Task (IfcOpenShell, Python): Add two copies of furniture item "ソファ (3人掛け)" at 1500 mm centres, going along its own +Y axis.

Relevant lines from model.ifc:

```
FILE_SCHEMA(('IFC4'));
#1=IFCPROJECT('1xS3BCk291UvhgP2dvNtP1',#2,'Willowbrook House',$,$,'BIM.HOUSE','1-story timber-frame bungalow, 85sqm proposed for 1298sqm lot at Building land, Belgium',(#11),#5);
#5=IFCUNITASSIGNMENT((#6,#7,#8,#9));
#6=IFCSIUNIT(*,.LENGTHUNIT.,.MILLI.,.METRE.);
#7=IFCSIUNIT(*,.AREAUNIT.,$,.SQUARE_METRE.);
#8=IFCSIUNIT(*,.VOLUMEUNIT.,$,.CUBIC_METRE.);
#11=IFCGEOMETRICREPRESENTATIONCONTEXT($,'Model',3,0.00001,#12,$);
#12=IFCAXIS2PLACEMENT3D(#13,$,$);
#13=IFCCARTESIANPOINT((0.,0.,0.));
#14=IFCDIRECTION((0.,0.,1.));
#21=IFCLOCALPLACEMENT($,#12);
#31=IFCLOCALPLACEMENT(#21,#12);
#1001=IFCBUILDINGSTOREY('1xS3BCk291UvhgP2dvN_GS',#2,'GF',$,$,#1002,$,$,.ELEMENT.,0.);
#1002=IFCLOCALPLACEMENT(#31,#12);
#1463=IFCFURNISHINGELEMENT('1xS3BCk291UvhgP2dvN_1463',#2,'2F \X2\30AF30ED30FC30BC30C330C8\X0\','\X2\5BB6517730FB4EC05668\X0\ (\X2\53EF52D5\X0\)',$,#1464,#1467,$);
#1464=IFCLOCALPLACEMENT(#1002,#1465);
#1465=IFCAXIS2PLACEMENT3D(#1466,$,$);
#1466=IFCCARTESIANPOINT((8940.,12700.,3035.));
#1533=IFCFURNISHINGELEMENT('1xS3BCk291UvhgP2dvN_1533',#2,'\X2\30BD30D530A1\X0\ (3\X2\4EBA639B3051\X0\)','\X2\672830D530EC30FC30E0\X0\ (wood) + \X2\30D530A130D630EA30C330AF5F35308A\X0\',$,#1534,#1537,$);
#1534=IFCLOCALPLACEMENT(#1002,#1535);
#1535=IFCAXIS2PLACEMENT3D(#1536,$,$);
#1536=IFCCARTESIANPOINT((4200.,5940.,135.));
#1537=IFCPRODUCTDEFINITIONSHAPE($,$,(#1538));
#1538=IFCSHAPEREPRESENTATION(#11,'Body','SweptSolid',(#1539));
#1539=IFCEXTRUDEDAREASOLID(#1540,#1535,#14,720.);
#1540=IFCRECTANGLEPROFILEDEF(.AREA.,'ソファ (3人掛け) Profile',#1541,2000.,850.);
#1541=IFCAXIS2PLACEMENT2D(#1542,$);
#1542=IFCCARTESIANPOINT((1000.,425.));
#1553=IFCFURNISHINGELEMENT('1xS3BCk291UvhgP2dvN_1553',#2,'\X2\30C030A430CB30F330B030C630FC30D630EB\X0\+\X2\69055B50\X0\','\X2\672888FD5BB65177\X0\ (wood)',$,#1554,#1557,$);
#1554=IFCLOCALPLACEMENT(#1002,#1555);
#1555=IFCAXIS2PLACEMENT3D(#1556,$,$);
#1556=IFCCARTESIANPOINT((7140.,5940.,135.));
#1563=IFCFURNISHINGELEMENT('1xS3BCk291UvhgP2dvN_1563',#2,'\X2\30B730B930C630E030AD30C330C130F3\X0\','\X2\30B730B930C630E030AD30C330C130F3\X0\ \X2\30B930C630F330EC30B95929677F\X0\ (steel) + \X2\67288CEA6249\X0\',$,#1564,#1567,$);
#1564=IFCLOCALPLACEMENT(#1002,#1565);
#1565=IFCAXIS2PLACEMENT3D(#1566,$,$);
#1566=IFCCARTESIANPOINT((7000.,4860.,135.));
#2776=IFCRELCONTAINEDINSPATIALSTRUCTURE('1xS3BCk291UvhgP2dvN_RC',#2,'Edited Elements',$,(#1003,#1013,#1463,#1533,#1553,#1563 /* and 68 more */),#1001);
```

```python
import ifcopenshell
import ifcopenshell.api.geometry
import ifcopenshell.api.root
import ifcopenshell.util.element
import ifcopenshell.util.placement
import ifcopenshell.util.unit

model = ifcopenshell.open("model.ifc")
unit_scale = ifcopenshell.util.unit.calculate_unit_scale(model)


def reuse_history(source, copy):
    """copy_class also copies each property set's owner history, people and application; keep the originals."""
    for rel in copy.IsDefinedBy:
        if rel.is_a("IfcRelDefinesByProperties") and (history := rel.RelatingPropertyDefinition.OwnerHistory):
            rel.RelatingPropertyDefinition.OwnerHistory = source.OwnerHistory
            ifcopenshell.util.element.remove_deep2(model, history)


source = model.by_id(1533)
base = ifcopenshell.util.placement.get_local_placement(source.ObjectPlacement)
step = base[:3, 1] * 1.5 / unit_scale

for i in range(1, 3):
    copy = ifcopenshell.api.root.copy_class(model, product=source)
    copy.Representation = ifcopenshell.util.element.copy_deep(
        model, source.Representation, exclude=["IfcGeometricRepresentationContext", "IfcRepresentationMap"]
    )
    reuse_history(source, copy)
    matrix = base.copy()
    matrix[:3, 3] += i * step
    print("added at", matrix[:3, 3].round(3) + 0.0)
    ifcopenshell.api.geometry.edit_object_placement(model, product=copy, matrix=matrix, is_si=False)

model.write("model-out.ifc")
```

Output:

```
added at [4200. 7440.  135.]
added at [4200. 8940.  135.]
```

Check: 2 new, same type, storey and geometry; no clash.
